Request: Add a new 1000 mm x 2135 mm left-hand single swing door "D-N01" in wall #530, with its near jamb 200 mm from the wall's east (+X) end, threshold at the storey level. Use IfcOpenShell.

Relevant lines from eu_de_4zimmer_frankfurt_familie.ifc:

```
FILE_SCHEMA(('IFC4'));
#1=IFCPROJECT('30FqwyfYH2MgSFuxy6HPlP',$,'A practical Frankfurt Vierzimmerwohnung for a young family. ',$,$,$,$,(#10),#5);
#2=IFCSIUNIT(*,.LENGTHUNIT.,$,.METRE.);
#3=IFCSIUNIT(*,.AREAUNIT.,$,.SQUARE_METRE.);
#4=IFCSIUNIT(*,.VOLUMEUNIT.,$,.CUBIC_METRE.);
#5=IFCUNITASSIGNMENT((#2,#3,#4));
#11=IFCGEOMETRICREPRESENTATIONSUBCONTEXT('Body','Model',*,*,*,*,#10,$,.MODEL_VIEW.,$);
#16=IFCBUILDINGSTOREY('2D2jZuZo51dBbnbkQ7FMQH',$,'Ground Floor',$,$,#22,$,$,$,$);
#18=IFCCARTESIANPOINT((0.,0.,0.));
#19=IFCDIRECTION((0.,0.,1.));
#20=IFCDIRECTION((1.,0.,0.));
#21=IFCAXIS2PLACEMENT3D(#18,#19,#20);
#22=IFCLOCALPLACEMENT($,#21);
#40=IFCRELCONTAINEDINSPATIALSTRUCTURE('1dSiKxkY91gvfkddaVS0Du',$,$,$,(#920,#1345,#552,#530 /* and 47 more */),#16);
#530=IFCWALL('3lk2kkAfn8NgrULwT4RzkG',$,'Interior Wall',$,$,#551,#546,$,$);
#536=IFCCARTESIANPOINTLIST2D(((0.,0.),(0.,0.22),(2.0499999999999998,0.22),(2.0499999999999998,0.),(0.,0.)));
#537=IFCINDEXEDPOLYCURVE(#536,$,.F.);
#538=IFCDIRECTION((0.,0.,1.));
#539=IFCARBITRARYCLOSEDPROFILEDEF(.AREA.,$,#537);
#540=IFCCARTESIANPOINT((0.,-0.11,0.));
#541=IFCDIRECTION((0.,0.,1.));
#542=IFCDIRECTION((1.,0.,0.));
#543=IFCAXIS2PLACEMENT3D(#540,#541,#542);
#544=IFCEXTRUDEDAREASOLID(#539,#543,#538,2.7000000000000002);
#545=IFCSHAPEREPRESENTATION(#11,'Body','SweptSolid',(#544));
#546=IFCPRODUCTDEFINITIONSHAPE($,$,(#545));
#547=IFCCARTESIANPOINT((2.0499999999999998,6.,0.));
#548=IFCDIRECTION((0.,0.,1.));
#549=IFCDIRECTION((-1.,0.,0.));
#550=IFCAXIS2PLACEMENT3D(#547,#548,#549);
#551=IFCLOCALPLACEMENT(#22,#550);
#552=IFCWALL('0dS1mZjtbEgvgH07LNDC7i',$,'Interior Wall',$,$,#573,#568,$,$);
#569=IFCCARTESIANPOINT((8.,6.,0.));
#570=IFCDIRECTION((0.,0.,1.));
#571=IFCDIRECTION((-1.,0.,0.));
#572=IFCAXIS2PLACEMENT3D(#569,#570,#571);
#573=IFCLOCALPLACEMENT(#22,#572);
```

```python
import numpy as np
import ifcopenshell
import ifcopenshell.api.feature
import ifcopenshell.api.geometry
import ifcopenshell.api.root
import ifcopenshell.api.spatial
import ifcopenshell.geom
import ifcopenshell.util.element
import ifcopenshell.util.placement
import ifcopenshell.util.representation
import ifcopenshell.util.shape
import ifcopenshell.util.unit

model = ifcopenshell.open("eu_de_4zimmer_frankfurt_familie.ifc")
unit_scale = ifcopenshell.util.unit.calculate_unit_scale(model)
settings = ifcopenshell.geom.settings()


def volume(element):
    """Net volume in cubic metres, openings subtracted."""
    shape = ifcopenshell.geom.create_shape(settings, element)
    return ifcopenshell.util.shape.get_volume(shape.geometry)


wall = model.by_guid("3lk2kkAfn8NgrULwT4RzkG")
storey = ifcopenshell.util.element.get_container(wall, ifc_class="IfcBuildingStorey")
context = ifcopenshell.util.representation.get_context(model, "Model", "Body", "MODEL_VIEW")
before = volume(wall)

width, height, from_end, sill = 1, 2.135, 0.2, 0.0  # metres

# The wall runs along its own X axis, and the end named is its -X end.
wall_shape = ifcopenshell.geom.create_shape(settings, wall)
x, y, z = ifcopenshell.util.shape.get_vertices(wall_shape.geometry).T
start = x.min() + from_end
face, thickness = float(y.min()), float(y.max() - y.min())
wall_matrix = ifcopenshell.util.placement.get_local_placement(wall.ObjectPlacement)
level = ifcopenshell.util.placement.get_local_placement(storey.ObjectPlacement)[2, 3]


def in_wall(x, y):
    """Placement at x, y metres in the wall's axes, at sill height."""
    matrix = wall_matrix.copy()
    matrix[:, 3] = wall_matrix @ np.array([x / unit_scale, y / unit_scale, 0.0, 1.0])
    matrix[2, 3] = level + sill / unit_scale
    return matrix


# Opening: a box that overshoots both wall faces by 50 mm.
opening = ifcopenshell.api.root.create_entity(model, ifc_class="IfcOpeningElement", predefined_type="OPENING")
box = ifcopenshell.api.geometry.add_wall_representation(
    model, context=context, length=width, height=height, thickness=thickness + 0.1
)
ifcopenshell.api.geometry.assign_representation(model, product=opening, representation=box)
ifcopenshell.api.geometry.edit_object_placement(model, product=opening, matrix=in_wall(start, face - 0.05), is_si=False)
ifcopenshell.api.feature.add_feature(model, feature=opening, element=wall)

door = ifcopenshell.api.root.create_entity(model, ifc_class="IfcDoor", name="D-N01", predefined_type="DOOR")
door.OverallWidth, door.OverallHeight = width / unit_scale, height / unit_scale
door.OperationType = "SINGLE_SWING_LEFT"
body = ifcopenshell.api.geometry.add_door_representation(
    model,
    context=context,
    overall_width=door.OverallWidth,
    overall_height=door.OverallHeight,
    operation_type="SINGLE_SWING_LEFT",
    lining_properties={"LiningDepth": thickness / unit_scale, "ThresholdDepth": thickness / unit_scale},
)
ifcopenshell.api.geometry.assign_representation(model, product=door, representation=body)
ifcopenshell.api.spatial.assign_container(model, products=[door], relating_structure=storey)
ifcopenshell.api.feature.add_filling(model, opening=opening, element=door)

# The lining spans the wall, so the door starts at the wall face.
ifcopenshell.api.geometry.edit_object_placement(model, product=door, matrix=in_wall(start, face), is_si=False)

after = volume(wall)

print(f"wall volume {before:.3f} -> {after:.3f} m3")

model.write("eu_de_4zimmer_frankfurt_familie_v2.ifc")
```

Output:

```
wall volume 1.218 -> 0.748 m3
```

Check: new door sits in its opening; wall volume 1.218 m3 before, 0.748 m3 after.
